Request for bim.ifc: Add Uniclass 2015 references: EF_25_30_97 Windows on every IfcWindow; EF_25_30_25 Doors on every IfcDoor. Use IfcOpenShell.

First a look at what the model holds.

```python
import ifcopenshell

model = ifcopenshell.open("bim.ifc")
print(model.schema)
print("classifications:", [c.Name for c in model.by_type("IfcClassification")])
for ifc_class in ("IfcDoor", "IfcRoof", "IfcStair", "IfcWall", "IfcWindow"):
    print(ifc_class, len(model.by_type(ifc_class)))
```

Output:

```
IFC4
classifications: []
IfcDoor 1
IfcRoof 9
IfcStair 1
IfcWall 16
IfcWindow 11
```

```python
import ifcopenshell
import ifcopenshell.api.classification

model = ifcopenshell.open("bim.ifc")

system = ifcopenshell.api.classification.add_classification(model, classification="Uniclass 2015")

codes = {
    "IfcWindow": ("EF_25_30_97", "Windows"),
    "IfcDoor": ("EF_25_30_25", "Doors"),
}
for ifc_class, (code, name) in codes.items():
    products = model.by_type(ifc_class)
    ifcopenshell.api.classification.add_reference(
        model, products=products, classification=system, identification=code, name=name
    )
    print(code, len(products))

model.write("bim_updated.ifc")
```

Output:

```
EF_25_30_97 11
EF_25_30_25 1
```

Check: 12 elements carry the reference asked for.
